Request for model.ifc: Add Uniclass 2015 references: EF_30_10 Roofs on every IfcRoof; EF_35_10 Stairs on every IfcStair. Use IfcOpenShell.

First a look at what the model holds.

```python
import ifcopenshell

model = ifcopenshell.open("model.ifc")
print(model.schema)
print("classifications:", [c.Name for c in model.by_type("IfcClassification")])
for ifc_class in ("IfcDoor", "IfcRoof", "IfcStair", "IfcWall", "IfcWindow"):
    print(ifc_class, len(model.by_type(ifc_class)))
```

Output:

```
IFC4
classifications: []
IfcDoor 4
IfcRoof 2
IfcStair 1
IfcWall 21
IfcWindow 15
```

```python
import ifcopenshell
import ifcopenshell.api.classification

model = ifcopenshell.open("model.ifc")

system = ifcopenshell.api.classification.add_classification(model, classification="Uniclass 2015")

codes = {
    "IfcRoof": ("EF_30_10", "Roofs"),
    "IfcStair": ("EF_35_10", "Stairs"),
}
for ifc_class, (code, name) in codes.items():
    products = model.by_type(ifc_class)
    ifcopenshell.api.classification.add_reference(
        model, products=products, classification=system, identification=code, name=name
    )
    print(code, len(products))

model.write("model_updated.ifc")
```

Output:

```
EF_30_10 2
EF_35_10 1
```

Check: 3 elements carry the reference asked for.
